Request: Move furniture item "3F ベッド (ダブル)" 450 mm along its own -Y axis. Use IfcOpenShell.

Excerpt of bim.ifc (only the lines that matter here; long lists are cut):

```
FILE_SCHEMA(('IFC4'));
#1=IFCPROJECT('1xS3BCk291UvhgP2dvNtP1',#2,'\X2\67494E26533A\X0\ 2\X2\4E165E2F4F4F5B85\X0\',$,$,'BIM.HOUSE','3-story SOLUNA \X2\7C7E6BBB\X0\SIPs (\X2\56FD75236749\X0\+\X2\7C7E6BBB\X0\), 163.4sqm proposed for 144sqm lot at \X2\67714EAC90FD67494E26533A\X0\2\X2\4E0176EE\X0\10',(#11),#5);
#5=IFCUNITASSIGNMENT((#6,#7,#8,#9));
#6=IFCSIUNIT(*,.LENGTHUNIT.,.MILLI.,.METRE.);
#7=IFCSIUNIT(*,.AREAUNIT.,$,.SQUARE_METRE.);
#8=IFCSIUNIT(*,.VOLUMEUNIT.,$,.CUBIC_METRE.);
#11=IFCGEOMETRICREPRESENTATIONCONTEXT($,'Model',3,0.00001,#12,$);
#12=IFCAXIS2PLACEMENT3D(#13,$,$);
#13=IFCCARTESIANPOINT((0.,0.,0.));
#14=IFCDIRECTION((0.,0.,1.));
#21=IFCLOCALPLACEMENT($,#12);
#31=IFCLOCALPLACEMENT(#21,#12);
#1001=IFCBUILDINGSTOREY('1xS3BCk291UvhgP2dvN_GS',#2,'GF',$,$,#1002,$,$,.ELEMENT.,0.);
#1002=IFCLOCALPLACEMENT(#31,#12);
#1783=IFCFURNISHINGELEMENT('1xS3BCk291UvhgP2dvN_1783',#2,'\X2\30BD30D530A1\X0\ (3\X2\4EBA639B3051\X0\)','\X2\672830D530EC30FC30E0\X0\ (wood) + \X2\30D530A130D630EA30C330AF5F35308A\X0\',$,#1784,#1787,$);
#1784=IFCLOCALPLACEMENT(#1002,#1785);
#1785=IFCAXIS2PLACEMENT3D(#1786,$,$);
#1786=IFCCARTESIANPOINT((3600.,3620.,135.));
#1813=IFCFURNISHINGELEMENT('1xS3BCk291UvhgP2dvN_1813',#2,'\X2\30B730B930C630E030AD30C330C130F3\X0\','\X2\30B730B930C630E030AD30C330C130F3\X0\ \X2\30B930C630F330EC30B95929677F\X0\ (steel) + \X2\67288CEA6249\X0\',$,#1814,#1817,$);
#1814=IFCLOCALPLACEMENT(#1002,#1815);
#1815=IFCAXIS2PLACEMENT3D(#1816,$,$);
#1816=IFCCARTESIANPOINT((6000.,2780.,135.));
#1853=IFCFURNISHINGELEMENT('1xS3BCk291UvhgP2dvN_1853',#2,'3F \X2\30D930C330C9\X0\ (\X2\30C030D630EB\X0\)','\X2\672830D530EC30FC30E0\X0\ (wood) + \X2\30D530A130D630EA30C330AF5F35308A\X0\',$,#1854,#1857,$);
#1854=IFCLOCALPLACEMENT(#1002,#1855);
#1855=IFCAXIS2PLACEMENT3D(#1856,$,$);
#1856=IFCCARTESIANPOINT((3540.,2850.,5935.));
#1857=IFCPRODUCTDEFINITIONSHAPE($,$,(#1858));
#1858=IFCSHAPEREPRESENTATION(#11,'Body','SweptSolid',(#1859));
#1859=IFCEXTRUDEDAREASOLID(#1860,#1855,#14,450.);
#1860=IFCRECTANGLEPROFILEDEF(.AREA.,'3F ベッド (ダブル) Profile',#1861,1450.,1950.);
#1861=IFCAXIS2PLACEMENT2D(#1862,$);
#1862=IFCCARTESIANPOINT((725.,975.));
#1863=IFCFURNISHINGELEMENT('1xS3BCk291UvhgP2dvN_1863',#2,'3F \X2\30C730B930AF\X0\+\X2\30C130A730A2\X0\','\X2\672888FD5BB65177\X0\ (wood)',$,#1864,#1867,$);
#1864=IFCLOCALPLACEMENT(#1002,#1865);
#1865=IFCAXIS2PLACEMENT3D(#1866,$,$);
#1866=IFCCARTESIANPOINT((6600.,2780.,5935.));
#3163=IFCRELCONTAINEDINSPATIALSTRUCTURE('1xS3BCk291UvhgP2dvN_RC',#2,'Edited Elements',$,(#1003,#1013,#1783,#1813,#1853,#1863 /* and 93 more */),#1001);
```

```python
import ifcopenshell
import ifcopenshell.api.geometry
import ifcopenshell.util.placement
import ifcopenshell.util.unit

model = ifcopenshell.open("bim.ifc")
unit_scale = ifcopenshell.util.unit.calculate_unit_scale(model)

item = model.by_guid("1xS3BCk291UvhgP2dvN_1853")
matrix = ifcopenshell.util.placement.get_local_placement(item.ObjectPlacement)
matrix[:3, 3] -= matrix[:3, 1] * 0.45 / unit_scale
ifcopenshell.api.geometry.edit_object_placement(model, product=item, matrix=matrix, is_si=False)

print(ifcopenshell.util.placement.get_local_placement(item.ObjectPlacement).round(3) + 0.0)

model.write("bim_v2.ifc")
```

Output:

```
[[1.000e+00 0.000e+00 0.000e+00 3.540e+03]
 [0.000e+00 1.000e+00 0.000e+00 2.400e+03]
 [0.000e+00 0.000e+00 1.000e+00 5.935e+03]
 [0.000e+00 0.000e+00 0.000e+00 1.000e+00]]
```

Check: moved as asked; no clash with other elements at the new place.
